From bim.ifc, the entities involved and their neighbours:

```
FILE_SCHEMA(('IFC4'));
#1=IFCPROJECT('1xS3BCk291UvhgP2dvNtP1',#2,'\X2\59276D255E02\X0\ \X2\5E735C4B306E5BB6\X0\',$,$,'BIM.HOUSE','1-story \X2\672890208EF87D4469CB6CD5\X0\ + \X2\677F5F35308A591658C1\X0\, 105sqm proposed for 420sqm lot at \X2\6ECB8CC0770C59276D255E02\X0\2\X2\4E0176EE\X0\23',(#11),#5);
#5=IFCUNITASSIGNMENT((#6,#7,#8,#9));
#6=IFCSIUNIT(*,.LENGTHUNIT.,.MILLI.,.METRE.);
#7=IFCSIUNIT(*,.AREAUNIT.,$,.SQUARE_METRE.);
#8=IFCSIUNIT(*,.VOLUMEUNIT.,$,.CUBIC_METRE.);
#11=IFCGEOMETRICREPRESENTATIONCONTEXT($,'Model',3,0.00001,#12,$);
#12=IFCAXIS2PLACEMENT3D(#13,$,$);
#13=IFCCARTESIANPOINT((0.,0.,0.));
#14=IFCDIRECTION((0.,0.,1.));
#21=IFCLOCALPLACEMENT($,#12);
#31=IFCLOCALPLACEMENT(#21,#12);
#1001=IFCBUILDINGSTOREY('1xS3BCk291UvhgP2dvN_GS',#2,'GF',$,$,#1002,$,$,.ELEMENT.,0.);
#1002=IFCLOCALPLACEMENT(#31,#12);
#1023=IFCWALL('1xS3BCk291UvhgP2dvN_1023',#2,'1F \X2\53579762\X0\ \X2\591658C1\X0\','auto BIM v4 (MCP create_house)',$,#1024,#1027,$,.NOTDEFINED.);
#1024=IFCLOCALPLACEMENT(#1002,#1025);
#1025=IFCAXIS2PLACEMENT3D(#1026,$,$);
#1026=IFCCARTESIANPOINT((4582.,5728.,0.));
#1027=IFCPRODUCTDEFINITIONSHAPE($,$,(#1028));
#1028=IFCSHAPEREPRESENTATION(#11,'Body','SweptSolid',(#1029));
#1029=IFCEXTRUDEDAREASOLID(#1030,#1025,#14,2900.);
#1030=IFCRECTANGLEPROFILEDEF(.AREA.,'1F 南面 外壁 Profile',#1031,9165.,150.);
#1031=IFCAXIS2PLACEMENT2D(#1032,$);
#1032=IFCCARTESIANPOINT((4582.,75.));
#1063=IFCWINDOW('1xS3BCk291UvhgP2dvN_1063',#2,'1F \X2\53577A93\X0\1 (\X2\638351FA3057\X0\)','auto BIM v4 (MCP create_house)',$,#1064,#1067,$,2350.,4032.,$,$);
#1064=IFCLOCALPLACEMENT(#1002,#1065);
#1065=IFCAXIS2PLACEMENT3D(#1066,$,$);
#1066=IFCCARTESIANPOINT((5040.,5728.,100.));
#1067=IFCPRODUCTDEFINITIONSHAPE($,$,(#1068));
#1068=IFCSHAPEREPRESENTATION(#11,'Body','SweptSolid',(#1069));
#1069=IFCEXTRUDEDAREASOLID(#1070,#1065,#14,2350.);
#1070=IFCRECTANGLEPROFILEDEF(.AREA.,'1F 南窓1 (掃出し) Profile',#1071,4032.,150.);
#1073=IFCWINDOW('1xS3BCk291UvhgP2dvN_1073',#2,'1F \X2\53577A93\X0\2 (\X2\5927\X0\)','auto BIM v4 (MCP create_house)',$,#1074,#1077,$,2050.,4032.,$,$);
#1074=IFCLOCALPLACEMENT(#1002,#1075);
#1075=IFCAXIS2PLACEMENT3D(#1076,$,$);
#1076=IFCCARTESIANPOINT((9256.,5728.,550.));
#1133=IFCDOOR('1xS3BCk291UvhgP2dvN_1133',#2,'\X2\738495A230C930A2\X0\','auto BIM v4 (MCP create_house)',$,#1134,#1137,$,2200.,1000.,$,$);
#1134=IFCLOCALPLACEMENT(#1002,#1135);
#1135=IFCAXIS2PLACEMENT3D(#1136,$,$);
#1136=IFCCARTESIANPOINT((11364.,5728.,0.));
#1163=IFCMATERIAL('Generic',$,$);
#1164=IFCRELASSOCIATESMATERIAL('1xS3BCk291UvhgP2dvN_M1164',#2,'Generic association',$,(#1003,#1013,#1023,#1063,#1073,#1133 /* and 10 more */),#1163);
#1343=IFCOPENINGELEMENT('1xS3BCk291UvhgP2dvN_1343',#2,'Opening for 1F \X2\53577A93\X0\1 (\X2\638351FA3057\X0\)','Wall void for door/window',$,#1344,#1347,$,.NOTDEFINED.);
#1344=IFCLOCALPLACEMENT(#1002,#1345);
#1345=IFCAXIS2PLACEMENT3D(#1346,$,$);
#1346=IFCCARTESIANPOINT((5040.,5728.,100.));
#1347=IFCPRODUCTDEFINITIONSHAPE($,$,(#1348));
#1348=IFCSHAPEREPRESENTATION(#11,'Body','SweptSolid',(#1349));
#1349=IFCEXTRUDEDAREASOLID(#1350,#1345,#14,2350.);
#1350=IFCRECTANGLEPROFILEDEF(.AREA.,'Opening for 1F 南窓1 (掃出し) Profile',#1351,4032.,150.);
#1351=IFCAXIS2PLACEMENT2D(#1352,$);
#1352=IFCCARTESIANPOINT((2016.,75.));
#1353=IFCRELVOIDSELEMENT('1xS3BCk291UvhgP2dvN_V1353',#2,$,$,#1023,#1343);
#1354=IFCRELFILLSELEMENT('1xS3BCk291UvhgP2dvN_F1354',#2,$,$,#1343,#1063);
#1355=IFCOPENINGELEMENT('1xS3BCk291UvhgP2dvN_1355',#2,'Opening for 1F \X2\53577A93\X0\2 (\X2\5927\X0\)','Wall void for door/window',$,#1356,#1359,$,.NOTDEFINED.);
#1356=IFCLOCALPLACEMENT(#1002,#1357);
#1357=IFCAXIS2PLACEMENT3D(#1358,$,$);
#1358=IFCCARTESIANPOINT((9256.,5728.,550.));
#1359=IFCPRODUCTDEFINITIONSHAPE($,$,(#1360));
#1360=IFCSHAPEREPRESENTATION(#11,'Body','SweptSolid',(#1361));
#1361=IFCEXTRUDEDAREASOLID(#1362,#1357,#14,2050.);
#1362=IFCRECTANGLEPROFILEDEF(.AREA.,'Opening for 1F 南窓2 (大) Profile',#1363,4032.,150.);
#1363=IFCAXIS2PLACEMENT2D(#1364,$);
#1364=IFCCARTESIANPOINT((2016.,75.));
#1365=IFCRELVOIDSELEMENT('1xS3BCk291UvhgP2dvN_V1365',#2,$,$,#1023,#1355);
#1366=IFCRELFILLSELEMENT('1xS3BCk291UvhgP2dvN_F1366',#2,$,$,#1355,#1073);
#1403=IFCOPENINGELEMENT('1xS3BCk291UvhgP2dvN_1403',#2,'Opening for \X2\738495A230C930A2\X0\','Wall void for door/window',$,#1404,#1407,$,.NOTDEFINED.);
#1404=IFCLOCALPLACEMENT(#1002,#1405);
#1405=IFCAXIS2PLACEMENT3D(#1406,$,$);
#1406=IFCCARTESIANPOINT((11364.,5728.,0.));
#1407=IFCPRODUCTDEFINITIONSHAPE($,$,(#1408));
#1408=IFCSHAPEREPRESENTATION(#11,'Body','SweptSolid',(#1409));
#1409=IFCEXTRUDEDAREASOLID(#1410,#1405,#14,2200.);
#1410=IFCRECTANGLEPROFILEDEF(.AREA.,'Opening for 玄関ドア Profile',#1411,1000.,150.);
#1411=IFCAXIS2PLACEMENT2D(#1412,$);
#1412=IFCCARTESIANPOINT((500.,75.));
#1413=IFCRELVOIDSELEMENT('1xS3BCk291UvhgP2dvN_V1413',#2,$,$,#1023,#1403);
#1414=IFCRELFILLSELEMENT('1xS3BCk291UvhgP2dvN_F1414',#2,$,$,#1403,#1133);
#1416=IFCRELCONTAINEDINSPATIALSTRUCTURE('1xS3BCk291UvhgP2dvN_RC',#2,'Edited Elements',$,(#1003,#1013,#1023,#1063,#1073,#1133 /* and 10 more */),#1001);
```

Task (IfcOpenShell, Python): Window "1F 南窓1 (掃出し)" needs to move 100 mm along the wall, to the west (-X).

```python
import ifcopenshell
import ifcopenshell.api.geometry
import ifcopenshell.util.placement
import ifcopenshell.util.unit

model = ifcopenshell.open("bim.ifc")
unit_scale = ifcopenshell.util.unit.calculate_unit_scale(model)

window = model.by_guid("1xS3BCk291UvhgP2dvN_1063")
opening = window.FillsVoids[0].RelatingOpeningElement
wall = opening.VoidsElements[0].RelatingBuildingElement

wall_matrix = ifcopenshell.util.placement.get_local_placement(wall.ObjectPlacement)
shift = wall_matrix[:3, 0] * -0.1 / unit_scale
before = ifcopenshell.util.placement.get_local_placement(window.ObjectPlacement)[:3, 3].copy()

# The window is not placed relative to its opening, so move both.
for product in (opening, window):
    matrix = ifcopenshell.util.placement.get_local_placement(product.ObjectPlacement)
    matrix[:3, 3] += shift
    ifcopenshell.api.geometry.edit_object_placement(model, product=product, matrix=matrix, is_si=False)

after = ifcopenshell.util.placement.get_local_placement(window.ObjectPlacement)[:3, 3]
print("window moved by", (after - before).round(3) + 0.0)

model.write("bim_rev.ifc")
```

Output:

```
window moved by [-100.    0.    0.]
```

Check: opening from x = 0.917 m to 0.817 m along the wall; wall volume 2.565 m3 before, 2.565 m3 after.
